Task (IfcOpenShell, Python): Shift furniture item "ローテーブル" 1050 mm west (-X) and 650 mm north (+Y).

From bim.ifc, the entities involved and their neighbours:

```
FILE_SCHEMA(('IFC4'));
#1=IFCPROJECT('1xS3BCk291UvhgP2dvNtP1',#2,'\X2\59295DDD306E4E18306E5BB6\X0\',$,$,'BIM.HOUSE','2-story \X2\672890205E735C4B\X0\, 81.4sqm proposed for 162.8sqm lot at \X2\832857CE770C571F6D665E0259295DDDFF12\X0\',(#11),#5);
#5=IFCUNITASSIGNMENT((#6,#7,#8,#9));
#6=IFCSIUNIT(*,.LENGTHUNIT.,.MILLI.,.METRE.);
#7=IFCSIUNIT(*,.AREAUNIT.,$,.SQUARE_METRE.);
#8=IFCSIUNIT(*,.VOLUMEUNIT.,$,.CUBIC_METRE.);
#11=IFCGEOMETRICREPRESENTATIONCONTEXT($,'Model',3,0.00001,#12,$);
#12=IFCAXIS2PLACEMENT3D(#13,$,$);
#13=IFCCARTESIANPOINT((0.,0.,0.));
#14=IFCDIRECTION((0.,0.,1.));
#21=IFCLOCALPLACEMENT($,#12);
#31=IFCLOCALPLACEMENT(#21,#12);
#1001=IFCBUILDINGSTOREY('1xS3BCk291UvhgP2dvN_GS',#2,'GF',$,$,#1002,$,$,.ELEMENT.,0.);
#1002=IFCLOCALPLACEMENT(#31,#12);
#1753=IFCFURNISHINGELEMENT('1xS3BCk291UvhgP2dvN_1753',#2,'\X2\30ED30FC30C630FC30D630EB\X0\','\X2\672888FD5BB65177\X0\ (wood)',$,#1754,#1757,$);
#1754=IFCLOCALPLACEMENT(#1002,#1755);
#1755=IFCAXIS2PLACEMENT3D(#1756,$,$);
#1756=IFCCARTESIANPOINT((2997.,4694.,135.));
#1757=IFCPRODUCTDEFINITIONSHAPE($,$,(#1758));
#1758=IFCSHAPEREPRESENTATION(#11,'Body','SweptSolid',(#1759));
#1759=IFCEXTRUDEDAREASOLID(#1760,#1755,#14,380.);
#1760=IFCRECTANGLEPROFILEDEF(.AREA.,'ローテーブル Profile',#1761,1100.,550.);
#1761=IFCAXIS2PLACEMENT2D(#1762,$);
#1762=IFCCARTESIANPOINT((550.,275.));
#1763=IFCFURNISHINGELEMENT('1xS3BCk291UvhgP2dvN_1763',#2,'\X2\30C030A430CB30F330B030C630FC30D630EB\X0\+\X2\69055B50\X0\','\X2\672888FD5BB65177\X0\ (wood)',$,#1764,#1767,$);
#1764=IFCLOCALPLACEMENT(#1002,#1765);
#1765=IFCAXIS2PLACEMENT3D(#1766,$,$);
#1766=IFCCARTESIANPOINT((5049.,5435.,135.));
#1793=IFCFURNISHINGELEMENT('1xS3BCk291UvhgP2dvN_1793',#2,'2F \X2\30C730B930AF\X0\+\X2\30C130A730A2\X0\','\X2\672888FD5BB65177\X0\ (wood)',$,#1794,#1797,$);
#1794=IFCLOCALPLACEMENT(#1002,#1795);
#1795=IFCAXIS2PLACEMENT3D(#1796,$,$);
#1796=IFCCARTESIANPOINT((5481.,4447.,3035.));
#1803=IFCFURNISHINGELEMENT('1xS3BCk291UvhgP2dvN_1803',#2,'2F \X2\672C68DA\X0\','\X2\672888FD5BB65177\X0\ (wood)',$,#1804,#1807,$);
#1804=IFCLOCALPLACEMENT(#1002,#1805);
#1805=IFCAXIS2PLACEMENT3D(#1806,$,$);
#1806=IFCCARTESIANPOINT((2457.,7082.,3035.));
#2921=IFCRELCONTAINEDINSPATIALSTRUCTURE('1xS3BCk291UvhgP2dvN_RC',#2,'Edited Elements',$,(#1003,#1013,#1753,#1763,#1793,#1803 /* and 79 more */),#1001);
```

```python
import ifcopenshell
import ifcopenshell.api.geometry
import ifcopenshell.util.placement
import ifcopenshell.util.unit

model = ifcopenshell.open("bim.ifc")
unit_scale = ifcopenshell.util.unit.calculate_unit_scale(model)

item = model.by_guid("1xS3BCk291UvhgP2dvN_1753")
matrix = ifcopenshell.util.placement.get_local_placement(item.ObjectPlacement)
matrix[0, 3] -= 1.05 / unit_scale
matrix[1, 3] += 0.65 / unit_scale
ifcopenshell.api.geometry.edit_object_placement(model, product=item, matrix=matrix, is_si=False)

print(ifcopenshell.util.placement.get_local_placement(item.ObjectPlacement).round(3) + 0.0)

model.write("bim_updated.ifc")
```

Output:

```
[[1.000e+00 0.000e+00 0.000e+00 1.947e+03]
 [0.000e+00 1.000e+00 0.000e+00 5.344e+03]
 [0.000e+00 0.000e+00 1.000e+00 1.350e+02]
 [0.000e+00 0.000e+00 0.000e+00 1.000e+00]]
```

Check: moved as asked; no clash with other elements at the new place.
